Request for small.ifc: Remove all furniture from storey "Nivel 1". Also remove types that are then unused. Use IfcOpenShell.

First a look at what the model holds.

```python
import ifcopenshell
import ifcopenshell.util.element

model = ifcopenshell.open("small.ifc")
print(model.schema)
storey = next(s for s in model.by_type("IfcBuildingStorey") if s.Name == "Nivel 1")
furniture = [e for e in ifcopenshell.util.element.get_decomposition(storey) if e.is_a("IfcFurnishingElement")]
seen = {}
for e in furniture:
    element_type = ifcopenshell.util.element.get_type(e)
    name = element_type.Name if element_type not in (None, e) else None
    seen[name] = seen.get(name, 0) + 1
for name, count in sorted(seen.items(), key=str):
    print(count, "x", name)
```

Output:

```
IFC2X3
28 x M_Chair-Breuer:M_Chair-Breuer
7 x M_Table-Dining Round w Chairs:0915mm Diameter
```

```python
import ifcopenshell
import ifcopenshell.api.root
import ifcopenshell.util.element

model = ifcopenshell.open("small.ifc")

storey = next(s for s in model.by_type("IfcBuildingStorey") if s.Name == "Nivel 1")
furniture = [e for e in ifcopenshell.util.element.get_decomposition(storey) if e.is_a("IfcFurnishingElement")]
types = {ifcopenshell.util.element.get_type(e) for e in furniture} - {None, *furniture}

for e in furniture:
    ifcopenshell.api.root.remove_product(model, product=e)
print(len(furniture), "removed")

unused = [t for t in types if not ifcopenshell.util.element.get_types(t)]
for t in unused:
    ifcopenshell.api.root.remove_product(model, product=t)
print(len(unused), "unused types removed")

model.write("small_rev.ifc")
```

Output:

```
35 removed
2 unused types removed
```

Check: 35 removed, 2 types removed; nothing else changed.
